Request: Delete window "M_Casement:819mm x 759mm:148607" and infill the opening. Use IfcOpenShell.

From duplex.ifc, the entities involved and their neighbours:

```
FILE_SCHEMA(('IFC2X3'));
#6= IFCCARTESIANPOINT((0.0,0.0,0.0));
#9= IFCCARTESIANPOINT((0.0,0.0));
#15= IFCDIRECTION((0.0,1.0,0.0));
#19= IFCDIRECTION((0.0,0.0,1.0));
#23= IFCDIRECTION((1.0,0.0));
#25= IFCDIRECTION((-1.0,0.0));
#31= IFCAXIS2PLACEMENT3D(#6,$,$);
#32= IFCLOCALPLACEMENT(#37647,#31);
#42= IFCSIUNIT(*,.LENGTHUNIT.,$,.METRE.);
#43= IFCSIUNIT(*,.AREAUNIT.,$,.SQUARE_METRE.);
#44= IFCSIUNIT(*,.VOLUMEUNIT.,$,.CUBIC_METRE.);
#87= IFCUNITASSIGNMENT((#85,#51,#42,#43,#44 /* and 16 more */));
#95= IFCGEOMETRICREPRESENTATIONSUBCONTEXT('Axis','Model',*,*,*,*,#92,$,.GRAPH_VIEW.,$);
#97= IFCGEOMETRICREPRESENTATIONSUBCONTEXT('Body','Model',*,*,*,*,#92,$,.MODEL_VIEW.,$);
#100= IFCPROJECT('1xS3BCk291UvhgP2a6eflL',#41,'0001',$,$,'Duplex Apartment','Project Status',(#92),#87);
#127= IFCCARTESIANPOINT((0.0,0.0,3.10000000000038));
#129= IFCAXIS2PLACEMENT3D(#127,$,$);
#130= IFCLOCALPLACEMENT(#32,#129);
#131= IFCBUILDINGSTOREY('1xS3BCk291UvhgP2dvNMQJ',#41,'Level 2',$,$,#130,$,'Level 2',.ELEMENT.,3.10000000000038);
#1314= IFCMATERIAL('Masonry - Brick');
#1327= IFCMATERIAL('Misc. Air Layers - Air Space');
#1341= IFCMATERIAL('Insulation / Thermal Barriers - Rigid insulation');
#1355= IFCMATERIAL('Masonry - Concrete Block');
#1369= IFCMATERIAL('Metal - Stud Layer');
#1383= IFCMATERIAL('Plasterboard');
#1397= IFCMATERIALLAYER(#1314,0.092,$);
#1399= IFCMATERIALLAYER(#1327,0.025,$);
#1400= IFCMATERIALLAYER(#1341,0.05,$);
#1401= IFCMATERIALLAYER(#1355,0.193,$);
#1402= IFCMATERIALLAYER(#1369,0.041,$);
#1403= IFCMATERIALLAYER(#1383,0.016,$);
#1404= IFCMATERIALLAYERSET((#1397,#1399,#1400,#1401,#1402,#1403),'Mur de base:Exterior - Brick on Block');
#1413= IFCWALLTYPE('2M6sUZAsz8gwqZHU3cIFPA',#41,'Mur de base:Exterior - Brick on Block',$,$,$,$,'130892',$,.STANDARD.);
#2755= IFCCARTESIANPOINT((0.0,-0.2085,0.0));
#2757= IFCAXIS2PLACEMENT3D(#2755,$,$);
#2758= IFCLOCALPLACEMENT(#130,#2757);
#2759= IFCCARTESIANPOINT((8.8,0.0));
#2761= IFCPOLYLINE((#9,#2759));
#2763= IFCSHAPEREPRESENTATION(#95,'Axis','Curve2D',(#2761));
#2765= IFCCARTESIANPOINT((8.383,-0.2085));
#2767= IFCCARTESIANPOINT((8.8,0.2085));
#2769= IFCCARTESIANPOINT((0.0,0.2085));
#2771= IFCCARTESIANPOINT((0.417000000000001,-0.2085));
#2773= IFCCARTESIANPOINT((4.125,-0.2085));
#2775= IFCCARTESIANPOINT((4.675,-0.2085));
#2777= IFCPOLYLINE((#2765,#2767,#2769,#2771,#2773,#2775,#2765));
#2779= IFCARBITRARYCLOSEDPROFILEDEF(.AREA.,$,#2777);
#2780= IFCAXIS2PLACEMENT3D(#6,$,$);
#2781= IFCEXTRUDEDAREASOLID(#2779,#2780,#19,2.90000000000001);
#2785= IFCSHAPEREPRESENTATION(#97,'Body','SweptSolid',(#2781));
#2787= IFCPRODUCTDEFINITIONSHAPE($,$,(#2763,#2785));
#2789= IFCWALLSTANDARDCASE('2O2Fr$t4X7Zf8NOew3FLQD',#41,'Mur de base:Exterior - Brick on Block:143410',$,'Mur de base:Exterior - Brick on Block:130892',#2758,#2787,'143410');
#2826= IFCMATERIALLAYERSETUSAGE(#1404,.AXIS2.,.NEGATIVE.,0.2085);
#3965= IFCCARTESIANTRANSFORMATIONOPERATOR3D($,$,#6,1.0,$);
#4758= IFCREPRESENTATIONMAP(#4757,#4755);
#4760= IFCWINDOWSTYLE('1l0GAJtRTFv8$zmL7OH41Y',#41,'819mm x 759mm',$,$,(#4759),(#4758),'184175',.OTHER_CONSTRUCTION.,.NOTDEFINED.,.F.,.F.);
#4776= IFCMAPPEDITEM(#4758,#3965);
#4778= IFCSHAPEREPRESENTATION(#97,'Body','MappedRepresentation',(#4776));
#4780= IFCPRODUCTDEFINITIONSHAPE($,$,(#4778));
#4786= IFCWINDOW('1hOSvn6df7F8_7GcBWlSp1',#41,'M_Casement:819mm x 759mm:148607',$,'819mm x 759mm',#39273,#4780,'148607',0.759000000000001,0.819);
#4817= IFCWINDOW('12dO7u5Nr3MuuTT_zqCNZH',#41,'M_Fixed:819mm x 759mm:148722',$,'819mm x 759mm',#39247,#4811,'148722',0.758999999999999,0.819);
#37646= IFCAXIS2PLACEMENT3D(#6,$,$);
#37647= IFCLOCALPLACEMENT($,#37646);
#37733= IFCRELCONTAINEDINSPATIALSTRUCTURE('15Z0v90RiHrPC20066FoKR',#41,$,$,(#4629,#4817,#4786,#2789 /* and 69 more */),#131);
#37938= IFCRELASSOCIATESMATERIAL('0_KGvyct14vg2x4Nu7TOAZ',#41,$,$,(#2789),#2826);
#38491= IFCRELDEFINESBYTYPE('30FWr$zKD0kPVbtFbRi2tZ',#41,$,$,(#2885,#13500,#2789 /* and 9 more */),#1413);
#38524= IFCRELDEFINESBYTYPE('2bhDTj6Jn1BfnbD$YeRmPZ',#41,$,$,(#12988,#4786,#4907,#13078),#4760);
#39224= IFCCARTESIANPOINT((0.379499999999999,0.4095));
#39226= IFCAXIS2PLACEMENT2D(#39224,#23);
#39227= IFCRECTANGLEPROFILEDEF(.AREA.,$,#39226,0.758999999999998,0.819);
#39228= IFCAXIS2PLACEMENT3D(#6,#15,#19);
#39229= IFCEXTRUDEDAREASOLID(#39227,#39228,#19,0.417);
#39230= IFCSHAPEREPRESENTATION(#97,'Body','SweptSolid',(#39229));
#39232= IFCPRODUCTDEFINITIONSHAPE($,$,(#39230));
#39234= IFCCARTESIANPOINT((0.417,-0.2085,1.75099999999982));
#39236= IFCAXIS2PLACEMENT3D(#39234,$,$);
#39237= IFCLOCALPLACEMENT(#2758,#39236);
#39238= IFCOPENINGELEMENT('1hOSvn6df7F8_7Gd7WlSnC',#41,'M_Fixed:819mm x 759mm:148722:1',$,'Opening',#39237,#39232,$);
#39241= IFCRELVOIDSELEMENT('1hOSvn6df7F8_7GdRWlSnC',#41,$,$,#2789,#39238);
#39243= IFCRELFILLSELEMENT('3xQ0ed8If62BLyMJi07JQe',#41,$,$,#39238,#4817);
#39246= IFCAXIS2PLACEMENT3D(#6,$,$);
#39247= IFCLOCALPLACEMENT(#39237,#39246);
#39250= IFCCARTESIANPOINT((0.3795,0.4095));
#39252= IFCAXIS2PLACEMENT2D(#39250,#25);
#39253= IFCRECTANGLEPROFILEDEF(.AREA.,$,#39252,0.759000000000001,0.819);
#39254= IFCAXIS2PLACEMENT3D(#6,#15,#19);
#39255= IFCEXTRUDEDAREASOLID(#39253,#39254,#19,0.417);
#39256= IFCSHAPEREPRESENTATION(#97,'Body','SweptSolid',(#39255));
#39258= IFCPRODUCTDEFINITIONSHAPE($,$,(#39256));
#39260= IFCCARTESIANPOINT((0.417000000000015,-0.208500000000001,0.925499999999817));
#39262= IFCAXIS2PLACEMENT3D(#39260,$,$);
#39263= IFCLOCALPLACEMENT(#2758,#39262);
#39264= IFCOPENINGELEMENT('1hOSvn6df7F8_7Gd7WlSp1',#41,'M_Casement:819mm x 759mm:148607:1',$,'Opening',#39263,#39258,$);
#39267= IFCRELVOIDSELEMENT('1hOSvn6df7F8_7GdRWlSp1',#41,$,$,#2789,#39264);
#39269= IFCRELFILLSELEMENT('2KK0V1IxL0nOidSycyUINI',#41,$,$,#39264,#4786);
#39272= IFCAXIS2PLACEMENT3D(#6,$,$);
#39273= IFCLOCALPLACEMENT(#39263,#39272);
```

```python
import ifcopenshell
import ifcopenshell.api.feature
import ifcopenshell.api.root
import ifcopenshell.geom
import ifcopenshell.util.shape

model = ifcopenshell.open("duplex.ifc")
settings = ifcopenshell.geom.settings()


def volume(element):
    """Net volume in cubic metres, openings subtracted."""
    shape = ifcopenshell.geom.create_shape(settings, element)
    return ifcopenshell.util.shape.get_volume(shape.geometry)


window = model.by_guid("1hOSvn6df7F8_7GcBWlSp1")
opening = window.FillsVoids[0].RelatingOpeningElement
wall = opening.VoidsElements[0].RelatingBuildingElement
before = volume(wall)

ifcopenshell.api.root.remove_product(model, product=window)
ifcopenshell.api.feature.remove_feature(model, feature=opening)

after = volume(wall)

print(f"wall volume {before:.3f} -> {after:.3f} m3")

model.write("duplex_rev.ifc")
```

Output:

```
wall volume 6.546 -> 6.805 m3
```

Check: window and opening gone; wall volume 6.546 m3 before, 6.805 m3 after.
